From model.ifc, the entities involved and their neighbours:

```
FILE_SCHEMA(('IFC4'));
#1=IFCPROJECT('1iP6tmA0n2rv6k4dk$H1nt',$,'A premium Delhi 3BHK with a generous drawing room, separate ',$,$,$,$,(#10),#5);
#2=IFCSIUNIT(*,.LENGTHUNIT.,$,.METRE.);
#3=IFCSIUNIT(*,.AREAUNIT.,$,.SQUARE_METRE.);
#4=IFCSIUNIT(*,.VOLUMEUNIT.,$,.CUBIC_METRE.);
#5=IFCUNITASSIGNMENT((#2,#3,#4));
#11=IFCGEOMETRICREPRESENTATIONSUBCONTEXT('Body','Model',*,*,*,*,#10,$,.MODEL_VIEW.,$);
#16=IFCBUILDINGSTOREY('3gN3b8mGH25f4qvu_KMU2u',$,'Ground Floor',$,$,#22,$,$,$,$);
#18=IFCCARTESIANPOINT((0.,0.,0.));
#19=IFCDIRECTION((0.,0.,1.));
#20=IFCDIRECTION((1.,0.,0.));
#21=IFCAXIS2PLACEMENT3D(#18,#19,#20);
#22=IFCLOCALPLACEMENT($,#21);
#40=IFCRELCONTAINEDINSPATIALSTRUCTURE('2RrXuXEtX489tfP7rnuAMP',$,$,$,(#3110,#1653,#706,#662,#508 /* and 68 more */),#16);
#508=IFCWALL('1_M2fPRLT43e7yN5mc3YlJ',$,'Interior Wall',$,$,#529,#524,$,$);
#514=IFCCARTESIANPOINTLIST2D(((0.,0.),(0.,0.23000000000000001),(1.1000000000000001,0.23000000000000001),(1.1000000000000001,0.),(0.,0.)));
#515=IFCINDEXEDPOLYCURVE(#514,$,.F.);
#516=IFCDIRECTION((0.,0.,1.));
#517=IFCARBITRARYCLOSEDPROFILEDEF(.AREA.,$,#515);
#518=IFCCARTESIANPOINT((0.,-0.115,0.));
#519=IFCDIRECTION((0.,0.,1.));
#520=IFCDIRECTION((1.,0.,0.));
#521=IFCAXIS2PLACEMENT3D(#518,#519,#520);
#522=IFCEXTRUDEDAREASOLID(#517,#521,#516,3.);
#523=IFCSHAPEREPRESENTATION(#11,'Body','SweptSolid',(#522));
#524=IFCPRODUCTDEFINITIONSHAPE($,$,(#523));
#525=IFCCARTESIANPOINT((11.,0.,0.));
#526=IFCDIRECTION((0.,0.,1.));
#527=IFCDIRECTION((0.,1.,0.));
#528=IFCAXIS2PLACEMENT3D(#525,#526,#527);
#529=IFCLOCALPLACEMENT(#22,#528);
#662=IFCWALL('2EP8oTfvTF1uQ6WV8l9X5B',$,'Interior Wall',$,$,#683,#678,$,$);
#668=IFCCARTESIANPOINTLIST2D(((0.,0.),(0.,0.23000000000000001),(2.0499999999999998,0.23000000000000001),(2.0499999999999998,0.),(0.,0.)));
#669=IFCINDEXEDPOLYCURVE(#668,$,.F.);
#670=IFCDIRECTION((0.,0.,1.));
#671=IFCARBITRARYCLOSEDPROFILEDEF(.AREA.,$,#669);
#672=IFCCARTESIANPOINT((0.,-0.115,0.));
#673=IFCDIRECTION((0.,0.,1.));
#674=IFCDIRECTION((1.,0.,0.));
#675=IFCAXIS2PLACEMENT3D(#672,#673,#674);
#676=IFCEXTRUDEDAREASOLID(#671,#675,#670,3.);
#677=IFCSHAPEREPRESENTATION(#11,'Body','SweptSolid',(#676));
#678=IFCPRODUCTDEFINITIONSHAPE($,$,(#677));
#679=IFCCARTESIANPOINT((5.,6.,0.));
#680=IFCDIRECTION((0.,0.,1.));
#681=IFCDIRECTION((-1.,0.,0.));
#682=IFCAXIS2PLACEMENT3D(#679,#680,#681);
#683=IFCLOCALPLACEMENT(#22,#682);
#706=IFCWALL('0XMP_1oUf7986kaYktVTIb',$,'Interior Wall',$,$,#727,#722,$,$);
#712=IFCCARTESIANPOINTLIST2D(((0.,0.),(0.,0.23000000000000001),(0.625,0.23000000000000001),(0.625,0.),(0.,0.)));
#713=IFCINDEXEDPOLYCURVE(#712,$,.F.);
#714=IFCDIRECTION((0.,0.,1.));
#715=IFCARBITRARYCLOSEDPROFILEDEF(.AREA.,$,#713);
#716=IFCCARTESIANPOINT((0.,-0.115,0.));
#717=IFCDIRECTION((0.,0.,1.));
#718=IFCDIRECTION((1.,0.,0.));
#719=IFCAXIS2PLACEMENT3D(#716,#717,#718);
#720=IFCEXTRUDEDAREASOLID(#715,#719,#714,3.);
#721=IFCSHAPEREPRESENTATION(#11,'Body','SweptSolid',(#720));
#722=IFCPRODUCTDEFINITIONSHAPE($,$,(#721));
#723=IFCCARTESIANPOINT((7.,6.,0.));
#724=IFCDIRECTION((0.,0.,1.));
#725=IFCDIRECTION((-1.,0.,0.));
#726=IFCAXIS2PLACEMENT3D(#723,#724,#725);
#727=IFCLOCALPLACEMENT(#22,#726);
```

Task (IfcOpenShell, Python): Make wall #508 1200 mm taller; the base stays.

```python
import ifcopenshell
import ifcopenshell.geom
import ifcopenshell.util.representation
import ifcopenshell.util.shape
import ifcopenshell.util.unit

model = ifcopenshell.open("model.ifc")
unit_scale = ifcopenshell.util.unit.calculate_unit_scale(model)
settings = ifcopenshell.geom.settings()


def volume(element):
    """Net volume in cubic metres, openings subtracted."""
    shape = ifcopenshell.geom.create_shape(settings, element)
    return ifcopenshell.util.shape.get_volume(shape.geometry)


wall = model.by_guid("1_M2fPRLT43e7yN5mc3YlJ")
before = volume(wall)

body = ifcopenshell.util.representation.get_representation(wall, "Model", "Body")
solid = body.Items[0]
old_height = solid.Depth
solid.Depth += 1.2 / unit_scale
after = volume(wall)

print(f"height {old_height:g} -> {solid.Depth:g}, volume {before:.3f} -> {after:.3f} m3")

model.write("model-out.ifc")
```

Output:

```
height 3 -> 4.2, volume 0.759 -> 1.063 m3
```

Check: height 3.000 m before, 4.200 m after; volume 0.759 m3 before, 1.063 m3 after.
